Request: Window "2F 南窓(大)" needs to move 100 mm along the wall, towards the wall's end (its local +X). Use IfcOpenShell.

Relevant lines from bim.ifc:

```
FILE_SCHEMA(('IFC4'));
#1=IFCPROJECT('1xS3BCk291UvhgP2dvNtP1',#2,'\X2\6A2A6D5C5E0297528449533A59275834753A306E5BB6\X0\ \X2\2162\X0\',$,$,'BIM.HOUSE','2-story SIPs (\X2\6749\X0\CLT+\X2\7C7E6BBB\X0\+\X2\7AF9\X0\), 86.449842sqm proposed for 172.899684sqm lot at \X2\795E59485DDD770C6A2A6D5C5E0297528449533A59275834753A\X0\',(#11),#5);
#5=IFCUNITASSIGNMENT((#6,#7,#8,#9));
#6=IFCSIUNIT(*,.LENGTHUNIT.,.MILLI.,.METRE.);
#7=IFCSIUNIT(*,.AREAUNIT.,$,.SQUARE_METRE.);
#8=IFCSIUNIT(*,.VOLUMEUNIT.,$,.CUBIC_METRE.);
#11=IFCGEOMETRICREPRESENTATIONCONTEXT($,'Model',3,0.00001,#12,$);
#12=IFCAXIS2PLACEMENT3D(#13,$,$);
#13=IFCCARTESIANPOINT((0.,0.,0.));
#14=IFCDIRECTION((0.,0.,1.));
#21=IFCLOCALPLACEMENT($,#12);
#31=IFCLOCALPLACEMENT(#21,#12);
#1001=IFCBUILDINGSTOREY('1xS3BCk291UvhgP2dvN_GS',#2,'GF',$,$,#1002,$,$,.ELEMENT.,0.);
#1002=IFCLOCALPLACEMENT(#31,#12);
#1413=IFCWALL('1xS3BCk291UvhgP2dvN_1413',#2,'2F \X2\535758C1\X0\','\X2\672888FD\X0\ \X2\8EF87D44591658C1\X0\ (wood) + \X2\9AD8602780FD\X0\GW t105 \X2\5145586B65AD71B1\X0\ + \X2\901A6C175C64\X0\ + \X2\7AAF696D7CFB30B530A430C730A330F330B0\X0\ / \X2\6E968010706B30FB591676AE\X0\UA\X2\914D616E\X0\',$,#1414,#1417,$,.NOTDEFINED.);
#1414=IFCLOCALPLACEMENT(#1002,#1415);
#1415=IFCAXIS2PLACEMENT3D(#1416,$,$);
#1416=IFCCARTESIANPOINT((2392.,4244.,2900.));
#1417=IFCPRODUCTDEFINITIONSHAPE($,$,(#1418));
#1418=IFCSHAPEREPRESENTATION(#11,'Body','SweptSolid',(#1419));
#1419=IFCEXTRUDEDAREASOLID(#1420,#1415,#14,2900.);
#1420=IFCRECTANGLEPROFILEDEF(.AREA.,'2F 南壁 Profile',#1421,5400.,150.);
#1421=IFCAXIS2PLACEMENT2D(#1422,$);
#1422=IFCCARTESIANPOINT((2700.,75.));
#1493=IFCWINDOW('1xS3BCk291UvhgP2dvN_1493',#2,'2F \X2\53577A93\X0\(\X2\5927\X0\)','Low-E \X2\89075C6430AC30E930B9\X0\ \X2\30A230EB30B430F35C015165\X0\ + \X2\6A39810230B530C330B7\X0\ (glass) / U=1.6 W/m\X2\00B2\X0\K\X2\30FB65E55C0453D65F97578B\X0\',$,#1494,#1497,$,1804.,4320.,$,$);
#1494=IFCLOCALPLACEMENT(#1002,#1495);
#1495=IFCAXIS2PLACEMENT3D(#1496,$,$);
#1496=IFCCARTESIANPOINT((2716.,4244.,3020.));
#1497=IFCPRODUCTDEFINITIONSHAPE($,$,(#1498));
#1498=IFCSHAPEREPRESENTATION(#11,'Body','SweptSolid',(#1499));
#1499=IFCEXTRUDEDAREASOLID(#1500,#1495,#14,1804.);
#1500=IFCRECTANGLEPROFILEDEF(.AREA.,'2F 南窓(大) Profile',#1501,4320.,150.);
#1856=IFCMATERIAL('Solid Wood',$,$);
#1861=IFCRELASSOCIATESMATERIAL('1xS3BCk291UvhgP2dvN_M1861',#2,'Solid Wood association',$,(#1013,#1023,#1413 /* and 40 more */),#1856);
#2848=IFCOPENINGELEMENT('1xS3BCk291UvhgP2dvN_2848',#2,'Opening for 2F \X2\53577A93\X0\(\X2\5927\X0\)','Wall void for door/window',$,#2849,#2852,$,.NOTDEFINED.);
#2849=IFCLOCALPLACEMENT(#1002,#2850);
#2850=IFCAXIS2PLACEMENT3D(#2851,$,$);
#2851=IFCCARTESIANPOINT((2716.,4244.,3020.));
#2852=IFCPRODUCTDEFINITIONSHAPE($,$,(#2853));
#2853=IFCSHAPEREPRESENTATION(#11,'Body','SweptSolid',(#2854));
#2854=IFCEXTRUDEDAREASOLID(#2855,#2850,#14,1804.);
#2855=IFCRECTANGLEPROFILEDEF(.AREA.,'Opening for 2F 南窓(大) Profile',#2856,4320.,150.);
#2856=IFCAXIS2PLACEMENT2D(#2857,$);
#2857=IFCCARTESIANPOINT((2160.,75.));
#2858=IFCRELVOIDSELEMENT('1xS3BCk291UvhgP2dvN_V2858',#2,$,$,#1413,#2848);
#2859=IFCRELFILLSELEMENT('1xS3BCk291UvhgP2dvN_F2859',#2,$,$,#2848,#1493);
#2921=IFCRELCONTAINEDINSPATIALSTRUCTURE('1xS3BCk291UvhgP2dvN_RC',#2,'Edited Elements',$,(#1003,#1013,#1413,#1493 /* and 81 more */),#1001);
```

```python
import ifcopenshell
import ifcopenshell.api.geometry
import ifcopenshell.util.placement
import ifcopenshell.util.unit

model = ifcopenshell.open("bim.ifc")
unit_scale = ifcopenshell.util.unit.calculate_unit_scale(model)

window = model.by_guid("1xS3BCk291UvhgP2dvN_1493")
opening = window.FillsVoids[0].RelatingOpeningElement
wall = opening.VoidsElements[0].RelatingBuildingElement

wall_matrix = ifcopenshell.util.placement.get_local_placement(wall.ObjectPlacement)
shift = wall_matrix[:3, 0] * 0.1 / unit_scale
before = ifcopenshell.util.placement.get_local_placement(window.ObjectPlacement)[:3, 3].copy()

# The window is not placed relative to its opening, so move both.
for product in (opening, window):
    matrix = ifcopenshell.util.placement.get_local_placement(product.ObjectPlacement)
    matrix[:3, 3] += shift
    ifcopenshell.api.geometry.edit_object_placement(model, product=product, matrix=matrix, is_si=False)

after = ifcopenshell.util.placement.get_local_placement(window.ObjectPlacement)[:3, 3]
print("window moved by", (after - before).round(3) + 0.0)

model.write("bim_rev.ifc")
```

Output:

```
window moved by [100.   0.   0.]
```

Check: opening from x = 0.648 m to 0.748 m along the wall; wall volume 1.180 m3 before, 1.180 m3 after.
